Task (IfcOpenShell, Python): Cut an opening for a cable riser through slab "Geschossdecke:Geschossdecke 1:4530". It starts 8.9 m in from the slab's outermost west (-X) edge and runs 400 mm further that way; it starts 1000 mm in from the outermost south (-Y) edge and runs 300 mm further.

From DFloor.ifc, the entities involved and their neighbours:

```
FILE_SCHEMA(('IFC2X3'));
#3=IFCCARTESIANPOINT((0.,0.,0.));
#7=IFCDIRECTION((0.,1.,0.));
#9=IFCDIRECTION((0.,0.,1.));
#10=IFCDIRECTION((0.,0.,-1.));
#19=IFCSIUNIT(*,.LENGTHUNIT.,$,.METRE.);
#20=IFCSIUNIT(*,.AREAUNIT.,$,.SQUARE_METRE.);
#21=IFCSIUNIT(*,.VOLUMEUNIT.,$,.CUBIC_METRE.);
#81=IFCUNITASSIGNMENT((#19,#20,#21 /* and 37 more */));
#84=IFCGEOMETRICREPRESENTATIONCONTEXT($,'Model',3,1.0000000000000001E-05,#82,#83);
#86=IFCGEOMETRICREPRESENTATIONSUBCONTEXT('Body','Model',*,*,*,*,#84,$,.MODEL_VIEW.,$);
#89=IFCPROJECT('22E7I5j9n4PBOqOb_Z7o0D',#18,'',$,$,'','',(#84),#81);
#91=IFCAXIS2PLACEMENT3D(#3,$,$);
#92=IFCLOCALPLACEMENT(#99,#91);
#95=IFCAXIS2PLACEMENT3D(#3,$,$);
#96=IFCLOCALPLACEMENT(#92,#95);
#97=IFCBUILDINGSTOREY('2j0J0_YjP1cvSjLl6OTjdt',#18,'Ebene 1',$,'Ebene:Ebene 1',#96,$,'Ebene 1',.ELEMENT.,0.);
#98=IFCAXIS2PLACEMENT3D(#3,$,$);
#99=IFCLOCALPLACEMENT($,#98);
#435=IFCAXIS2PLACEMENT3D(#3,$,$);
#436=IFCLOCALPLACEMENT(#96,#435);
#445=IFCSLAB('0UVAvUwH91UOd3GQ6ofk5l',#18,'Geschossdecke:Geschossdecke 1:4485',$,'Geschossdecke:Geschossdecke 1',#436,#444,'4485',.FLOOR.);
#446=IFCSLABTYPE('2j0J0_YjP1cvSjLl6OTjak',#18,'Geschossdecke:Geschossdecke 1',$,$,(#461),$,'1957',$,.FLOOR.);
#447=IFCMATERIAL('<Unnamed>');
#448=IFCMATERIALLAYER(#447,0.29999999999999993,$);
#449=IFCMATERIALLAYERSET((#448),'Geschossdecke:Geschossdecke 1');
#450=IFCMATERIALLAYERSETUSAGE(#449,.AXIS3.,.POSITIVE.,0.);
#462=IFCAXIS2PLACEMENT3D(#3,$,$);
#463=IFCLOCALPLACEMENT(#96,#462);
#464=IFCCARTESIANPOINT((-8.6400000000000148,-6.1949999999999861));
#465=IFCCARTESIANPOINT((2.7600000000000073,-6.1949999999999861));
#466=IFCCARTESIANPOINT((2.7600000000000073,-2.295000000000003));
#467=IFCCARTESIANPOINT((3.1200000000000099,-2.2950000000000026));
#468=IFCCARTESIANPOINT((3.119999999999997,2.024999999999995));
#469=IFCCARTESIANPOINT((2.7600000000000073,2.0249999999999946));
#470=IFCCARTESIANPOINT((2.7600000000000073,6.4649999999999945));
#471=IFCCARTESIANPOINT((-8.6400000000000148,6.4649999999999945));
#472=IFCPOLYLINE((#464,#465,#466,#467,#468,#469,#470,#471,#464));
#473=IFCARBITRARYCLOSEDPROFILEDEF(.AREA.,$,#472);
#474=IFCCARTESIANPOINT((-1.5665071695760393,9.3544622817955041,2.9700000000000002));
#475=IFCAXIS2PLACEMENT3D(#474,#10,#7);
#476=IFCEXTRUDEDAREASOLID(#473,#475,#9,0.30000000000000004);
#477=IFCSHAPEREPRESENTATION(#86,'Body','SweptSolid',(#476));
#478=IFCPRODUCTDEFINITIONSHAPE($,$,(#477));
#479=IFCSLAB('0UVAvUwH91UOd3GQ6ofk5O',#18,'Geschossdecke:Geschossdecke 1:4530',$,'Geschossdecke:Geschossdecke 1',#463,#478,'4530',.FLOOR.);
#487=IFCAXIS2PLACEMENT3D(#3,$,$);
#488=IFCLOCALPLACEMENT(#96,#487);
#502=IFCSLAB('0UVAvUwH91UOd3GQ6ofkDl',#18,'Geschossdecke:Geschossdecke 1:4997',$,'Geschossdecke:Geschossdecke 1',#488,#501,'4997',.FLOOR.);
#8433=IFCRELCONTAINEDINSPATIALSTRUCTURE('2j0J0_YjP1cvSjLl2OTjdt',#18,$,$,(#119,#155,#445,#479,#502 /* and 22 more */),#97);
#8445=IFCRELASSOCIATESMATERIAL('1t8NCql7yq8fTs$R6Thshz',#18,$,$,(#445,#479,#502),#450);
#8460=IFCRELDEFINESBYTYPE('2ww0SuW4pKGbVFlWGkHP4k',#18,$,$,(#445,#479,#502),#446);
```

```python
import numpy as np
import ifcopenshell
import ifcopenshell.api.feature
import ifcopenshell.api.geometry
import ifcopenshell.api.root
import ifcopenshell.geom
import ifcopenshell.util.placement
import ifcopenshell.util.representation
import ifcopenshell.util.shape
import ifcopenshell.util.unit

model = ifcopenshell.open("DFloor.ifc")
unit_scale = ifcopenshell.util.unit.calculate_unit_scale(model)
settings = ifcopenshell.geom.settings()


def volume(element):
    """Net volume in cubic metres, openings subtracted."""
    shape = ifcopenshell.geom.create_shape(settings, element)
    return ifcopenshell.util.shape.get_volume(shape.geometry)


slab = model.by_id(479)
before = volume(slab)

# Extent in the slab's own axes, in metres. The edges named are its -X and -Y sides.
slab_shape = ifcopenshell.geom.create_shape(settings, slab)
vertices = ifcopenshell.util.shape.get_vertices(slab_shape.geometry)
x_min, y_min, bottom = vertices.min(axis=0)
top = vertices[:, 2].max()

opening = ifcopenshell.api.root.create_entity(model, ifc_class="IfcOpeningElement", name="Cable riser opening")
context = ifcopenshell.util.representation.get_context(model, "Model", "Body", "MODEL_VIEW")
width, depth = 0.4, 0.3
outline = [(0.0, 0.0), (width, 0.0), (width, depth), (0.0, depth), (0.0, 0.0)]
# Overshoot both faces by 50 mm so the cut is clean.
shape = ifcopenshell.api.geometry.add_slab_representation(
    model, context=context, depth=top - bottom + 0.1, polyline=outline
)
ifcopenshell.api.geometry.assign_representation(model, product=opening, representation=shape)

matrix = ifcopenshell.util.placement.get_local_placement(slab.ObjectPlacement)
matrix[:, 3] = matrix @ np.append(np.array([x_min + 8.9, y_min + 1, bottom - 0.05]) / unit_scale, 1.0)
ifcopenshell.api.geometry.edit_object_placement(model, product=opening, matrix=matrix, is_si=False)
ifcopenshell.api.feature.add_feature(model, feature=opening, element=slab)

after = volume(slab)

print(f"slab volume {before:.3f} -> {after:.3f} m3")

model.write("DFloor-out.ifc")
```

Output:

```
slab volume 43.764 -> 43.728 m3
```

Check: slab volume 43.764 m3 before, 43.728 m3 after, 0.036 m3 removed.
